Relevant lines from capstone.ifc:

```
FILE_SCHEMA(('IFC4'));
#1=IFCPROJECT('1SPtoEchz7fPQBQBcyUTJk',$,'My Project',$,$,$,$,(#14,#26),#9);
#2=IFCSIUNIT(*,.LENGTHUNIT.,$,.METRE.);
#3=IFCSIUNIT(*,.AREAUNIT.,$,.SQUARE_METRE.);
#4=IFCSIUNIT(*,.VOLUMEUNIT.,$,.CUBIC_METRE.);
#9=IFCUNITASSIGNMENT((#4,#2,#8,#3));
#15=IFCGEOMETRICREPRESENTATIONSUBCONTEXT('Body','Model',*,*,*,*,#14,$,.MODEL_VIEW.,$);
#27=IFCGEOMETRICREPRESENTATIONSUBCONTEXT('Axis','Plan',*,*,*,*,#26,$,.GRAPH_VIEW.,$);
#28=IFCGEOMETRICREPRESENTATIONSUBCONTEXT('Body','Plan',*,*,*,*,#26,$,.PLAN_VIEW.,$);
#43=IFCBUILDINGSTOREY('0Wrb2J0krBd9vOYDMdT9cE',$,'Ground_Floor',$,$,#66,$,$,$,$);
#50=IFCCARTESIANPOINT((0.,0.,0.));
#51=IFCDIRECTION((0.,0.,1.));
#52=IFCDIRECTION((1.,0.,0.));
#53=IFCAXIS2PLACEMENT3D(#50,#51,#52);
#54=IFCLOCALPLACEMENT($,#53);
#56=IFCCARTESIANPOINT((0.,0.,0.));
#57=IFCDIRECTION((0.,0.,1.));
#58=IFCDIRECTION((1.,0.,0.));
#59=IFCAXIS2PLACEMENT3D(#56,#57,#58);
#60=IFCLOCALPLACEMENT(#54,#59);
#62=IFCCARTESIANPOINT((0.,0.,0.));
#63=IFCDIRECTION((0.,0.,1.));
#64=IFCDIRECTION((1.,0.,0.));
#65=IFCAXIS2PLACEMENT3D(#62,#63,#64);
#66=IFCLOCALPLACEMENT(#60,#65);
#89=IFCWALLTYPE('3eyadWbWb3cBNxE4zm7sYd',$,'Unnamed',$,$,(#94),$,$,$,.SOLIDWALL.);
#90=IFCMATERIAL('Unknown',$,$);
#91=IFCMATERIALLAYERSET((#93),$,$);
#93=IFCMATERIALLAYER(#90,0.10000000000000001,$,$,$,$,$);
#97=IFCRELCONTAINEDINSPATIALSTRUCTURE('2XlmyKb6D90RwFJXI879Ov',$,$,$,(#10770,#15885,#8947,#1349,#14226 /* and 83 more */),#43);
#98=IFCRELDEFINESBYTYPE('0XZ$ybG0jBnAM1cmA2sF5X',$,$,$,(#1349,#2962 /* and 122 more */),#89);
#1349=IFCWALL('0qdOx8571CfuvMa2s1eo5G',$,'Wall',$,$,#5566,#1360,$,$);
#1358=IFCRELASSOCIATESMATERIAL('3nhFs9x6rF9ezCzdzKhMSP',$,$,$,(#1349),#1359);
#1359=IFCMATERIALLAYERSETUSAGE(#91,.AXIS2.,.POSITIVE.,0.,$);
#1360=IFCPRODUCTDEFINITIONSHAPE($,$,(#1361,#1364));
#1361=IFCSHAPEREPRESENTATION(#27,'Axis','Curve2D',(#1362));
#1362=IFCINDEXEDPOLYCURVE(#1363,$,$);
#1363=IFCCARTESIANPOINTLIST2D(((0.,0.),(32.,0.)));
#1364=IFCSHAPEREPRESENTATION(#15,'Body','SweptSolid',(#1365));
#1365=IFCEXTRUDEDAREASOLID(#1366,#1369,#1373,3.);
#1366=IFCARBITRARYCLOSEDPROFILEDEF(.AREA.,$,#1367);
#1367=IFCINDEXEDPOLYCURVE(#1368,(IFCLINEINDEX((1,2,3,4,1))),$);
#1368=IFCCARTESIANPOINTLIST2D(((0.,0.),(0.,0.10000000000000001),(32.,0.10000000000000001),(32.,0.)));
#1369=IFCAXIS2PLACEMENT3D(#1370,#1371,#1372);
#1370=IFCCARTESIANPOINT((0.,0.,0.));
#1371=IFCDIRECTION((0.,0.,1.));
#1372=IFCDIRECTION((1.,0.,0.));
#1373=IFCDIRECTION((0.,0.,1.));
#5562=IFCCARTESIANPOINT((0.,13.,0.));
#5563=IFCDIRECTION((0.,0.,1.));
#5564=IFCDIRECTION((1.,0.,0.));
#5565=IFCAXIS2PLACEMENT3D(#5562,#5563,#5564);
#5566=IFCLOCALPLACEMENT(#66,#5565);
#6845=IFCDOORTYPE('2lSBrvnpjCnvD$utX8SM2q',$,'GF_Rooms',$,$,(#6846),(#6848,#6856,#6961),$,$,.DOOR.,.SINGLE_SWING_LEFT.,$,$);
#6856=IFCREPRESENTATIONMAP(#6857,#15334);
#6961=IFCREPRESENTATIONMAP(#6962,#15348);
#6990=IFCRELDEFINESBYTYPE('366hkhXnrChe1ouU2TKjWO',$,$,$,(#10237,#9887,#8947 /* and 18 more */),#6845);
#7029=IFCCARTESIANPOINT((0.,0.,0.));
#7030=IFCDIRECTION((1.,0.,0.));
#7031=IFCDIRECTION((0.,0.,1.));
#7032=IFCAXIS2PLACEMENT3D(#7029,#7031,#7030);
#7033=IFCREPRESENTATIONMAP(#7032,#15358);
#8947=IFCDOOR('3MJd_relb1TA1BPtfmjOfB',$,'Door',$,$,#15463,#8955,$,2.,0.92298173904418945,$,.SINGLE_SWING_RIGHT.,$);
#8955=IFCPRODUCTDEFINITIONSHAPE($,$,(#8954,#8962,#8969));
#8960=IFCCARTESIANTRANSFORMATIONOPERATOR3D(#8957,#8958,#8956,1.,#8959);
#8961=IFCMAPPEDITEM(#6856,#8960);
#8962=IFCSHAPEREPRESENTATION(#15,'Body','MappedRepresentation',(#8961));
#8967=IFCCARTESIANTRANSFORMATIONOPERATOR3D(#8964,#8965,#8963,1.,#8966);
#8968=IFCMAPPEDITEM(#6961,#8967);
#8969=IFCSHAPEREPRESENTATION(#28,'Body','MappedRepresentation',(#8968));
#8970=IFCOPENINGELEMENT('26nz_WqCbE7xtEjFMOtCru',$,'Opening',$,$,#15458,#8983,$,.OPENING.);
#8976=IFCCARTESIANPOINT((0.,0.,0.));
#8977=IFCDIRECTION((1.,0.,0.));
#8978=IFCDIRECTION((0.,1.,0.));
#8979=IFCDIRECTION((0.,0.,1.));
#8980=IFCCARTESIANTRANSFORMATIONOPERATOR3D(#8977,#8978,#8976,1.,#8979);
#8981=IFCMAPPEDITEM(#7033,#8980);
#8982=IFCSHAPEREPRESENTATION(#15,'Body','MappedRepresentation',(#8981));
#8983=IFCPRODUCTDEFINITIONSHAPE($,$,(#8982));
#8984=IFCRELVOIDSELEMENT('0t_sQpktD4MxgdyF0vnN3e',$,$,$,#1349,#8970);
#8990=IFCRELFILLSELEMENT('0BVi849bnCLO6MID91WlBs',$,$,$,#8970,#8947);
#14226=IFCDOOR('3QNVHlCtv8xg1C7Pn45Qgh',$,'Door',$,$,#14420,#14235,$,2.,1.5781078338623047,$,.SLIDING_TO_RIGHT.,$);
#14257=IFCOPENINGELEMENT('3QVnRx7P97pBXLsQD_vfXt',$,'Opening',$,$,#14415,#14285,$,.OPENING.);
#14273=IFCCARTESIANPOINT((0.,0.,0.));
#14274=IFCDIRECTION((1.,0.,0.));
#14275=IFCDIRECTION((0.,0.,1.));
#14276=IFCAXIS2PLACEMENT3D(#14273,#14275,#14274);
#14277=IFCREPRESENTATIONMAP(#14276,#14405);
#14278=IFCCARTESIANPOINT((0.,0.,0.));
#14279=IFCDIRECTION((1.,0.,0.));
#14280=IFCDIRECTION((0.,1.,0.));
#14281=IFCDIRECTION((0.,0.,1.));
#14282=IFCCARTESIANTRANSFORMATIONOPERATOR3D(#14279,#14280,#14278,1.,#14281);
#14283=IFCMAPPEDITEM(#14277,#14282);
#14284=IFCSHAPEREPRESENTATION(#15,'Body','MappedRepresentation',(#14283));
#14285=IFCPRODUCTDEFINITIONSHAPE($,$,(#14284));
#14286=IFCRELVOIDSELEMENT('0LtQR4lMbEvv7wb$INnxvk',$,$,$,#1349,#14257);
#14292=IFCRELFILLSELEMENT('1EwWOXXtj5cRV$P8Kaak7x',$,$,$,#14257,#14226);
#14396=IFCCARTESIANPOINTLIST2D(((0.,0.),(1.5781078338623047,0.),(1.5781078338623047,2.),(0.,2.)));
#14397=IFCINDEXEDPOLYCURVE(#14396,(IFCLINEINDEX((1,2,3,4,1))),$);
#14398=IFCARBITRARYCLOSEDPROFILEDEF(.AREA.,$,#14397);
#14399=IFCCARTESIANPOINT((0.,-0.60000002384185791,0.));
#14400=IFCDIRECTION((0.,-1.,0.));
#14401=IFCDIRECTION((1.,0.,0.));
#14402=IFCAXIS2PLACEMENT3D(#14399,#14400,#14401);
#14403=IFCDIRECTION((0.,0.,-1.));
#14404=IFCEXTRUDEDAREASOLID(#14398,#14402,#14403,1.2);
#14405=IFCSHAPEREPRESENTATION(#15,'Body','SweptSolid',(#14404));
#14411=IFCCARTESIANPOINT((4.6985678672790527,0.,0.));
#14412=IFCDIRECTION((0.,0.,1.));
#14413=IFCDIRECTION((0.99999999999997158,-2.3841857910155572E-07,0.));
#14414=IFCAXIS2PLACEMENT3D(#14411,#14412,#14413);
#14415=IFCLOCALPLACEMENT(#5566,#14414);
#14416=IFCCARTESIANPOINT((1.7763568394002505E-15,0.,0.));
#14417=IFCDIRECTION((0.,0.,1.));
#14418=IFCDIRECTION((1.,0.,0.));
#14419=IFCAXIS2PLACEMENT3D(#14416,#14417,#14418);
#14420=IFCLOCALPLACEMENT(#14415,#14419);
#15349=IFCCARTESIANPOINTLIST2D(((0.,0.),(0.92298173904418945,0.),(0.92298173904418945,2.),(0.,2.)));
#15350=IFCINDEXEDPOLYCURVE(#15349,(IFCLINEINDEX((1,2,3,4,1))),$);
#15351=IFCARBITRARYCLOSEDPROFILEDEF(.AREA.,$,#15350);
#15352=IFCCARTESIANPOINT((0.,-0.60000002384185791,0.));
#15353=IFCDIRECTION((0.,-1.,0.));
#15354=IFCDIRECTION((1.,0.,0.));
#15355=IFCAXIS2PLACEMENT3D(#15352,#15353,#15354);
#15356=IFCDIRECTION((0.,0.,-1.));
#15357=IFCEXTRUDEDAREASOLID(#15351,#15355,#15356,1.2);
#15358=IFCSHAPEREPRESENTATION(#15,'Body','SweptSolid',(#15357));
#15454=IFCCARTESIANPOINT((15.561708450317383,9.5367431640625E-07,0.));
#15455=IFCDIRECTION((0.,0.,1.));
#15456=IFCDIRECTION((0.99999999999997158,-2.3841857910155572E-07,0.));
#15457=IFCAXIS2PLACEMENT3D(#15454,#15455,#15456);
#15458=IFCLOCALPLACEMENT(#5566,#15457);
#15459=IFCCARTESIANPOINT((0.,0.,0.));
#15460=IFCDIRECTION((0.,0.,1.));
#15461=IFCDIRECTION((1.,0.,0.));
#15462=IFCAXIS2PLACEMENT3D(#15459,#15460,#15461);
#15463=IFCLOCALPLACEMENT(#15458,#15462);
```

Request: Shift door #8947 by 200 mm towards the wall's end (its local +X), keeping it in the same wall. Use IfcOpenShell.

```python
import ifcopenshell
import ifcopenshell.api.geometry
import ifcopenshell.util.placement
import ifcopenshell.util.unit

model = ifcopenshell.open("capstone.ifc")
unit_scale = ifcopenshell.util.unit.calculate_unit_scale(model)

door = model.by_guid("3MJd_relb1TA1BPtfmjOfB")
opening = door.FillsVoids[0].RelatingOpeningElement
wall = opening.VoidsElements[0].RelatingBuildingElement

wall_matrix = ifcopenshell.util.placement.get_local_placement(wall.ObjectPlacement)
shift = wall_matrix[:3, 0] * 0.2 / unit_scale
before = ifcopenshell.util.placement.get_local_placement(door.ObjectPlacement)[:3, 3].copy()

# The door is placed relative to its opening, so it follows when the opening moves.
matrix = ifcopenshell.util.placement.get_local_placement(opening.ObjectPlacement)
matrix[:3, 3] += shift
ifcopenshell.api.geometry.edit_object_placement(
    model, product=opening, matrix=matrix, is_si=False, should_transform_children=True
)

after = ifcopenshell.util.placement.get_local_placement(door.ObjectPlacement)[:3, 3]
print("door moved by", (after - before).round(3) + 0.0)

model.write("capstone_edited.ifc")
```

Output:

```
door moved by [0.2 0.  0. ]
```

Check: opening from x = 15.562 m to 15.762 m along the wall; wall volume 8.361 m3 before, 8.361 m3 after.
